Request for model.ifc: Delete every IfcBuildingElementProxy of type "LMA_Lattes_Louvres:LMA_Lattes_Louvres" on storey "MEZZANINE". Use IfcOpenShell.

First a look at what the model holds.

```python
import ifcopenshell
import ifcopenshell.util.element

model = ifcopenshell.open("model.ifc")
print(model.schema)
storey = next(s for s in model.by_type("IfcBuildingStorey") if s.Name == "MEZZANINE")
proxies = [e for e in ifcopenshell.util.element.get_decomposition(storey) if e.is_a("IfcBuildingElementProxy")]
seen = {}
for e in proxies:
    element_type = ifcopenshell.util.element.get_type(e)
    name = element_type.Name if element_type not in (None, e) else None
    seen[name] = seen.get(name, 0) + 1
for name, count in sorted(seen.items(), key=str):
    print(count, "x", name)
```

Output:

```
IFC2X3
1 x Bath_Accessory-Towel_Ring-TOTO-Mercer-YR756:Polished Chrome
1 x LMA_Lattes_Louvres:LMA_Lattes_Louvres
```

```python
import ifcopenshell
import ifcopenshell.api.root
import ifcopenshell.util.element

model = ifcopenshell.open("model.ifc")

storey = next(s for s in model.by_type("IfcBuildingStorey") if s.Name == "MEZZANINE")
proxies = [e for e in ifcopenshell.util.element.get_decomposition(storey) if e.is_a("IfcBuildingElementProxy")]
targets = [e for e in proxies if (t := ifcopenshell.util.element.get_type(e)) not in (None, e) and t.Name == "LMA_Lattes_Louvres:LMA_Lattes_Louvres"]

for e in targets:
    ifcopenshell.api.root.remove_product(model, product=e)
print(len(targets), "removed")

model.write("model_v2.ifc")
```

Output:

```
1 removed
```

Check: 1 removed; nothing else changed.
